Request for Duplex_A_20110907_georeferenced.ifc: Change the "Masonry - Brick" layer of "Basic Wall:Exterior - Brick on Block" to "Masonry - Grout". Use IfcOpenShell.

First a look at what the model holds.

```python
import ifcopenshell
import ifcopenshell.util.element

model = ifcopenshell.open("Duplex_A_20110907_georeferenced.ifc")
print(model.schema)
for layer_set in model.by_type("IfcMaterialLayerSet"):
    if layer_set.LayerSetName == "Basic Wall:Exterior - Brick on Block":
        for layer in layer_set.MaterialLayers:
            print(layer.id(), layer.Material and layer.Material.Name, layer.LayerThickness, sep=" | ")
        print(len(ifcopenshell.util.element.get_elements_by_material(model, layer_set)), "elements and types use it")
print(sorted(m.Name for m in model.by_type("IfcMaterial") if m.Name)[:60])
```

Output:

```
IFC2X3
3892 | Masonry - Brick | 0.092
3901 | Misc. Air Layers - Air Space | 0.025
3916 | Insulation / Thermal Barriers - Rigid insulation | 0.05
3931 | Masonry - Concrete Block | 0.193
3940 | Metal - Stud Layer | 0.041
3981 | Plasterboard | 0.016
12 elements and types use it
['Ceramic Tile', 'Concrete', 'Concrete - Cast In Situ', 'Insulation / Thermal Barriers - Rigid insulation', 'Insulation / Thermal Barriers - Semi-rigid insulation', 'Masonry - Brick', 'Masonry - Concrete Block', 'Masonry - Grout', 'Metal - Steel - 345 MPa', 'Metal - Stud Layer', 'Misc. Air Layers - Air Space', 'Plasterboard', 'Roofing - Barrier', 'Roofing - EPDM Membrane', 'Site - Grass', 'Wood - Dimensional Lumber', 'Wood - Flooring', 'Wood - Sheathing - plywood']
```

```python
import ifcopenshell
import ifcopenshell.api.material

model = ifcopenshell.open("Duplex_A_20110907_georeferenced.ifc")

layer_set = next(s for s in model.by_type("IfcMaterialLayerSet") if s.LayerSetName == "Basic Wall:Exterior - Brick on Block")
layer = next(l for l in layer_set.MaterialLayers if l.Material and l.Material.Name == "Masonry - Brick")
material = next(m for m in model.by_type("IfcMaterial") if m.Name == "Masonry - Grout")

# Point this one layer at the other material; renaming the old one would change it everywhere.
ifcopenshell.api.material.edit_layer(model, layer=layer, attributes={}, material=material)

print([l.Material.Name if l.Material else None for l in layer_set.MaterialLayers])

model.write("Duplex_A_20110907_georeferenced_edited.ifc")
```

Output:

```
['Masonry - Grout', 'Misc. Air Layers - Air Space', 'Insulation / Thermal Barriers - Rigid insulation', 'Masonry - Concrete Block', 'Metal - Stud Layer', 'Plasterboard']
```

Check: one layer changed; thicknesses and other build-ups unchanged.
